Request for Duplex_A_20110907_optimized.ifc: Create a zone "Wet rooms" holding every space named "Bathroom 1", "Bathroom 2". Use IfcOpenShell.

First a look at what the model holds.

```python
import ifcopenshell

model = ifcopenshell.open("Duplex_A_20110907_optimized.ifc")
print(model.schema)
seen = {}
for space in model.by_type("IfcSpace"):
    seen[space.LongName] = seen.get(space.LongName, 0) + 1
for name, count in sorted(seen.items(), key=str):
    print(count, "x", name)
print("zones:", [z.Name for z in model.by_type("IfcZone")][:20])
```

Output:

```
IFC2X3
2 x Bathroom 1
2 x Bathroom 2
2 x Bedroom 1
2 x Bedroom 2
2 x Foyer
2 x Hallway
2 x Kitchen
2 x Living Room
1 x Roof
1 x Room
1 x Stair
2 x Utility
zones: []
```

```python
import ifcopenshell
import ifcopenshell.api.group
import ifcopenshell.api.root

model = ifcopenshell.open("Duplex_A_20110907_optimized.ifc")

names = {"Bathroom 1", "Bathroom 2"}
spaces = [s for s in model.by_type("IfcSpace") if s.LongName in names]

zone = ifcopenshell.api.root.create_entity(model, ifc_class="IfcZone", name="Wet rooms")
ifcopenshell.api.group.assign_group(model, products=spaces, group=zone)
print(len(spaces), "spaces in", zone.Name)

model.write("Duplex_A_20110907_optimized_rev.ifc")
```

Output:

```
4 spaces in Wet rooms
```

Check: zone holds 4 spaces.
